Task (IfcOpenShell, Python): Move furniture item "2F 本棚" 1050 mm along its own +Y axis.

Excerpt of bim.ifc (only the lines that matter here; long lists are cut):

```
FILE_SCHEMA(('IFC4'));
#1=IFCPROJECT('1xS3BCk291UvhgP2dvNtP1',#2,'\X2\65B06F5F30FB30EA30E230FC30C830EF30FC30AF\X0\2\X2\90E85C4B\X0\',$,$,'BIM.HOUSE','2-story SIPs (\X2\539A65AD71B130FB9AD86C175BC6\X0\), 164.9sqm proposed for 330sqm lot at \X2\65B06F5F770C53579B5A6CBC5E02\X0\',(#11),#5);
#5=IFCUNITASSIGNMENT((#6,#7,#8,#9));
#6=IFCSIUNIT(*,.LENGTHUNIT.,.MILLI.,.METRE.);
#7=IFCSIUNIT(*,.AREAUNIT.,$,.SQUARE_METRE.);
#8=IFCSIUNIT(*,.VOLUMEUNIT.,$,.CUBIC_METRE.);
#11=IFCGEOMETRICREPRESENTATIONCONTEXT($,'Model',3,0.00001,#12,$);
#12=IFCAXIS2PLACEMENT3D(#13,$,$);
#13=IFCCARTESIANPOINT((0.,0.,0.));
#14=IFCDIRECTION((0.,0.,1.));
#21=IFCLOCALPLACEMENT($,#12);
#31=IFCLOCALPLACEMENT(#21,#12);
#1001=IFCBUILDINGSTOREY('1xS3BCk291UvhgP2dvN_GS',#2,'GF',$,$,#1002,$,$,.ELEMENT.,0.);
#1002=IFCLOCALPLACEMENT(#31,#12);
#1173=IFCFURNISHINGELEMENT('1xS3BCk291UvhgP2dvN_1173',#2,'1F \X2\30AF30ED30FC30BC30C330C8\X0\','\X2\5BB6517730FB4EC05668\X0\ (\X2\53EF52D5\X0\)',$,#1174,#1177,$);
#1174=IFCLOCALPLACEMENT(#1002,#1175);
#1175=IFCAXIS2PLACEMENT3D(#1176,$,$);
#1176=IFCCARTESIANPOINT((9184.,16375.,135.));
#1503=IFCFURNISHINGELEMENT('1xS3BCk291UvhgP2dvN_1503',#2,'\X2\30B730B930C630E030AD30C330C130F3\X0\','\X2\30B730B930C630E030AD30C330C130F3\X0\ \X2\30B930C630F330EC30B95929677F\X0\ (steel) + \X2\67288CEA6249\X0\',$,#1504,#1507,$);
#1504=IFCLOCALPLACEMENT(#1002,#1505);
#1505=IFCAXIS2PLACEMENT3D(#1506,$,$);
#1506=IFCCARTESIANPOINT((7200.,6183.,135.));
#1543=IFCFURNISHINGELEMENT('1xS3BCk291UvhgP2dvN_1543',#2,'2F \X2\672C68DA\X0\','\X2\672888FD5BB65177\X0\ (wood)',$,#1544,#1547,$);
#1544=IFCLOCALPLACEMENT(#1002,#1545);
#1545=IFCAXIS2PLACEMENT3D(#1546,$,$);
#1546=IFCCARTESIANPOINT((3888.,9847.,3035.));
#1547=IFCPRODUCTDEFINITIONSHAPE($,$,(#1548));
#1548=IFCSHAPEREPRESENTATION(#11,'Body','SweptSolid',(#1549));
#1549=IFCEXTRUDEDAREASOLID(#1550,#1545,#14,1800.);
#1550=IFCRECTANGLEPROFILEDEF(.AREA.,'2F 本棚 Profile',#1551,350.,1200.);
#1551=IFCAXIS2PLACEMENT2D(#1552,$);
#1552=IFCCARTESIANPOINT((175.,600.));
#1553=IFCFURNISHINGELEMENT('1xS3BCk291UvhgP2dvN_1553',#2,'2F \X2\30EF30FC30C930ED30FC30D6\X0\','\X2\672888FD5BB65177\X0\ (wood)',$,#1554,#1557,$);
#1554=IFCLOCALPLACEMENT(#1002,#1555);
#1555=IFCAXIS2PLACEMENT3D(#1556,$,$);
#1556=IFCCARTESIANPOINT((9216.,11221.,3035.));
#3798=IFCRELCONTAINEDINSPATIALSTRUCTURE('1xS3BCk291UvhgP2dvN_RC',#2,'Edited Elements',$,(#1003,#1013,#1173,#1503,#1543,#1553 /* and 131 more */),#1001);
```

```python
import ifcopenshell
import ifcopenshell.api.geometry
import ifcopenshell.util.placement
import ifcopenshell.util.unit

model = ifcopenshell.open("bim.ifc")
unit_scale = ifcopenshell.util.unit.calculate_unit_scale(model)

item = model.by_guid("1xS3BCk291UvhgP2dvN_1543")
matrix = ifcopenshell.util.placement.get_local_placement(item.ObjectPlacement)
matrix[:3, 3] += matrix[:3, 1] * 1.05 / unit_scale
ifcopenshell.api.geometry.edit_object_placement(model, product=item, matrix=matrix, is_si=False)

print(ifcopenshell.util.placement.get_local_placement(item.ObjectPlacement).round(3) + 0.0)

model.write("bim_updated.ifc")
```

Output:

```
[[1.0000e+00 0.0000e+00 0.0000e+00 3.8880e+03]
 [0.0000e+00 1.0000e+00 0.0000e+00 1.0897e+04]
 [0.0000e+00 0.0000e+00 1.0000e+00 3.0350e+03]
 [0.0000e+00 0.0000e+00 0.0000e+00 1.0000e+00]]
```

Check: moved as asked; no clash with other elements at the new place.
